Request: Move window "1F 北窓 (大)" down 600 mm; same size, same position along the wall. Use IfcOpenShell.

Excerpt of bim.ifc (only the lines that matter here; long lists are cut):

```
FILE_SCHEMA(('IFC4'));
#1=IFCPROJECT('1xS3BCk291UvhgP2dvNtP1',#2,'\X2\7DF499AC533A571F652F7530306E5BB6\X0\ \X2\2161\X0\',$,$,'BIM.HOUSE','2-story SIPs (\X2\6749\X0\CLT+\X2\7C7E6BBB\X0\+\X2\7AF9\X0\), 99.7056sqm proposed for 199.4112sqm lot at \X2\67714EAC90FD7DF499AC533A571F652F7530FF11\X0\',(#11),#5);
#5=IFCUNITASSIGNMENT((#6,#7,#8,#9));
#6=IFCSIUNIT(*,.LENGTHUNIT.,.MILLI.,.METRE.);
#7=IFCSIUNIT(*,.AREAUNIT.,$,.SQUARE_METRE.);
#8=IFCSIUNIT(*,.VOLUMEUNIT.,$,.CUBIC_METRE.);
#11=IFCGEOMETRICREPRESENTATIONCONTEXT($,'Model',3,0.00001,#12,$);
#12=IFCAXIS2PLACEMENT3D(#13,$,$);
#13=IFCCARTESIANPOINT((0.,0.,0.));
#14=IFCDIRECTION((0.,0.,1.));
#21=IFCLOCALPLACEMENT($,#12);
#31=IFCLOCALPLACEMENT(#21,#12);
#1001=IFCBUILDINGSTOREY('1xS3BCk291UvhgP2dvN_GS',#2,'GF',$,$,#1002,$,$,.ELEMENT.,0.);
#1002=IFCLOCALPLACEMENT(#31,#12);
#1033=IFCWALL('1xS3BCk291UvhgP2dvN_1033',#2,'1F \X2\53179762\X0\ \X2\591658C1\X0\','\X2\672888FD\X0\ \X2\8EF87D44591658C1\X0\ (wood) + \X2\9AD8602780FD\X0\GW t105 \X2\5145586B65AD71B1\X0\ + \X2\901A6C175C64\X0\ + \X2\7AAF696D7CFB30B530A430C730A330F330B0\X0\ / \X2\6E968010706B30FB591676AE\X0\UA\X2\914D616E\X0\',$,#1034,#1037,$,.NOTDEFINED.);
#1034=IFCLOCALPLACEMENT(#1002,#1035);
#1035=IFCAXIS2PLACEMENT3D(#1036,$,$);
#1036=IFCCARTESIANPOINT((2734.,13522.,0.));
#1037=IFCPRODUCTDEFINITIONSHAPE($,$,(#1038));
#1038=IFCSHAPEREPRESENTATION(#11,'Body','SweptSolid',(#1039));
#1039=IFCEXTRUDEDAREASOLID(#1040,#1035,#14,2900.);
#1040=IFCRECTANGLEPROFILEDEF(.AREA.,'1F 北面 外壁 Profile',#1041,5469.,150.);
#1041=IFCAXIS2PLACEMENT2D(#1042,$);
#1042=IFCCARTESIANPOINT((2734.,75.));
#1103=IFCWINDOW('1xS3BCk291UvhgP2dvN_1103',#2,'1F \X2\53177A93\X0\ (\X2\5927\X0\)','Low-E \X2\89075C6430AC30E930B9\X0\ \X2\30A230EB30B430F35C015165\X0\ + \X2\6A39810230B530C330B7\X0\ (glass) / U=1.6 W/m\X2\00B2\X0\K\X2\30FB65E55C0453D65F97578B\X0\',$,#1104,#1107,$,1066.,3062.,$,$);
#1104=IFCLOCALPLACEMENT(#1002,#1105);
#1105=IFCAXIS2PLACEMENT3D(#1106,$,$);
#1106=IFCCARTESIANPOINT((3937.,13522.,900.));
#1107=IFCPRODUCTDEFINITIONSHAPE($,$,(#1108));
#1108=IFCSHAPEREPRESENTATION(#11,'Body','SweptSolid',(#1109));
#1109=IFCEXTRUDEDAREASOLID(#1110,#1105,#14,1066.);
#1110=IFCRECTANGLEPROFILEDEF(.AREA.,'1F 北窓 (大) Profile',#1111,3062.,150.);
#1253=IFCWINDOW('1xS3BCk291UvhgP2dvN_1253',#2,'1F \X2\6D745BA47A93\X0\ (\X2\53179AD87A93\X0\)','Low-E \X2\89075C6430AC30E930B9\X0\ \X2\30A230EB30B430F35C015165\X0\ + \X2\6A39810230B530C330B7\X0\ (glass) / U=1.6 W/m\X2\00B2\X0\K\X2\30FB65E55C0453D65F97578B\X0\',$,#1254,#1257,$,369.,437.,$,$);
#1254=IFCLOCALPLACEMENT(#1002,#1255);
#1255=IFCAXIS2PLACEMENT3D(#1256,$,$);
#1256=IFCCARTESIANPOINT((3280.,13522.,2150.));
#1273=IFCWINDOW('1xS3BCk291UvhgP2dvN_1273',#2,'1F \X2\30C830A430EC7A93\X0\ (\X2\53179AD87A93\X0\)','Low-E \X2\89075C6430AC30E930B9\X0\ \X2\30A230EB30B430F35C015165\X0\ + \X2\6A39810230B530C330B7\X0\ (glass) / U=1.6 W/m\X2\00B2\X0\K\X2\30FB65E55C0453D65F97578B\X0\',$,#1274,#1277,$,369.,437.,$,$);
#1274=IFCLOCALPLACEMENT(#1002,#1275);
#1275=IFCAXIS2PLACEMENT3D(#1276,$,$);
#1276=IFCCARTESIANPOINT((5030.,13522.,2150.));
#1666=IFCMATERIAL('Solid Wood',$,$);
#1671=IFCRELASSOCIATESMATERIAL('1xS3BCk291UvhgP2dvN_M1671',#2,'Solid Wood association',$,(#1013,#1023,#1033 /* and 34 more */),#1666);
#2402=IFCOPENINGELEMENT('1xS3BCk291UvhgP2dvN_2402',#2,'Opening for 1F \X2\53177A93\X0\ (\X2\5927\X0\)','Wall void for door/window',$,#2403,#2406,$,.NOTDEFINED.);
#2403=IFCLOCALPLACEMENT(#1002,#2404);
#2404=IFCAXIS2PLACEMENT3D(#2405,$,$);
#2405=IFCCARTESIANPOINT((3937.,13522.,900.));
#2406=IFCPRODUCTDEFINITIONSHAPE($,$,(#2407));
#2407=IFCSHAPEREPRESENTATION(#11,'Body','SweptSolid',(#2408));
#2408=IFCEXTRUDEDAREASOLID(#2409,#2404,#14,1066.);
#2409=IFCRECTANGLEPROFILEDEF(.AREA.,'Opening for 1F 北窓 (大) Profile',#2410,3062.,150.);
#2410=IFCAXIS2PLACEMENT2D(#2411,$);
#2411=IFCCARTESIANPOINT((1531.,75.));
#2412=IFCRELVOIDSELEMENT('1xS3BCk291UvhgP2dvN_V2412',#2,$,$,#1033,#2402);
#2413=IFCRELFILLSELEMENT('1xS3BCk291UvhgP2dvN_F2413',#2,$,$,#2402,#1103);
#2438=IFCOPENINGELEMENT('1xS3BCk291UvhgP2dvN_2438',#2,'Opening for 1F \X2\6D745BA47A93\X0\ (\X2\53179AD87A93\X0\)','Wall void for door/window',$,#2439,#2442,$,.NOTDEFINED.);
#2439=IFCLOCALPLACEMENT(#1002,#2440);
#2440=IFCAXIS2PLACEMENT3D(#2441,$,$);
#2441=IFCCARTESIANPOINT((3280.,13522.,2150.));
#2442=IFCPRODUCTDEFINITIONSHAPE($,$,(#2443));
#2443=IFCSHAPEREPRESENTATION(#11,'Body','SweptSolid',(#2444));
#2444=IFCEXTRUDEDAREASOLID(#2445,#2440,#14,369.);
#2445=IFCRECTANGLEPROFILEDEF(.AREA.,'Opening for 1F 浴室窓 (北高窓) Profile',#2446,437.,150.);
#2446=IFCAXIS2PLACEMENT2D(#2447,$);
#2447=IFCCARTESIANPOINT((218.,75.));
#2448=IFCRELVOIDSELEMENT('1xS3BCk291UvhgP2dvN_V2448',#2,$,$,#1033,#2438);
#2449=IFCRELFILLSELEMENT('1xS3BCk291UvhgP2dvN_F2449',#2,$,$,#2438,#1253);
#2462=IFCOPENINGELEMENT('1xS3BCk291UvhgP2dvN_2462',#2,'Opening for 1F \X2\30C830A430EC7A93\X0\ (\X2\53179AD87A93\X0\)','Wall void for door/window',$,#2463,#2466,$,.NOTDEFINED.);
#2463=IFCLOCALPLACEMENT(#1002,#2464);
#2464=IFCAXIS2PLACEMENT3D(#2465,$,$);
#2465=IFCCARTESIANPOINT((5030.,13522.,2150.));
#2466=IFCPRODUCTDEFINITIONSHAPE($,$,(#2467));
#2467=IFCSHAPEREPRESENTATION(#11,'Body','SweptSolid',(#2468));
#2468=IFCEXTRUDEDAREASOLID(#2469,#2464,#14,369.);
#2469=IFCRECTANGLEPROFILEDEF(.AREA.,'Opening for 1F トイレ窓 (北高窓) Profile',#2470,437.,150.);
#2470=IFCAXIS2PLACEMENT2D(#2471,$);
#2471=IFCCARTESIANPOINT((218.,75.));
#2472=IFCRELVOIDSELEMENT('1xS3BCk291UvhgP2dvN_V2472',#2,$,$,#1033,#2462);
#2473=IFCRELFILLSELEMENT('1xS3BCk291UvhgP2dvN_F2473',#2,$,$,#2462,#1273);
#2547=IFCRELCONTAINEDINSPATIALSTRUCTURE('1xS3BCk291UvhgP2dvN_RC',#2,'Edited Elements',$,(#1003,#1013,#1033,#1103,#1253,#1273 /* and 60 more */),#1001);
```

```python
import numpy as np
import ifcopenshell
import ifcopenshell.api.geometry
import ifcopenshell.util.placement
import ifcopenshell.util.unit

model = ifcopenshell.open("bim.ifc")
unit_scale = ifcopenshell.util.unit.calculate_unit_scale(model)

window = model.by_guid("1xS3BCk291UvhgP2dvN_1103")
opening = window.FillsVoids[0].RelatingOpeningElement
dz = -600.0

shift = np.array([0.0, 0.0, dz])
# The window is not placed relative to its opening, so move both.
for product in (opening, window):
    matrix = ifcopenshell.util.placement.get_local_placement(product.ObjectPlacement)
    matrix[:3, 3] += shift
    ifcopenshell.api.geometry.edit_object_placement(model, product=product, matrix=matrix, is_si=False)

print(f"moved by {dz * unit_scale:+.3f} m")

model.write("bim_updated.ifc")
```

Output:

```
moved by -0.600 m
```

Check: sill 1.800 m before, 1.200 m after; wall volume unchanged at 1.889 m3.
